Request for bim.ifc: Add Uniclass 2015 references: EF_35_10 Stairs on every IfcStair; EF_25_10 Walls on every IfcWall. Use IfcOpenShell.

First a look at what the model holds.

```python
import ifcopenshell

model = ifcopenshell.open("bim.ifc")
print(model.schema)
print("classifications:", [c.Name for c in model.by_type("IfcClassification")])
for ifc_class in ("IfcDoor", "IfcRoof", "IfcStair", "IfcWall", "IfcWindow"):
    print(ifc_class, len(model.by_type(ifc_class)))
```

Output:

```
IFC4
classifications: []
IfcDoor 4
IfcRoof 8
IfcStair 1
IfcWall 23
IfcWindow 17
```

```python
import ifcopenshell
import ifcopenshell.api.classification

model = ifcopenshell.open("bim.ifc")

system = ifcopenshell.api.classification.add_classification(model, classification="Uniclass 2015")

codes = {
    "IfcStair": ("EF_35_10", "Stairs"),
    "IfcWall": ("EF_25_10", "Walls"),
}
for ifc_class, (code, name) in codes.items():
    products = model.by_type(ifc_class)
    ifcopenshell.api.classification.add_reference(
        model, products=products, classification=system, identification=code, name=name
    )
    print(code, len(products))

model.write("bim_edited.ifc")
```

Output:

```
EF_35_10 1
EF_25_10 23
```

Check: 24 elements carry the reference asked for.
